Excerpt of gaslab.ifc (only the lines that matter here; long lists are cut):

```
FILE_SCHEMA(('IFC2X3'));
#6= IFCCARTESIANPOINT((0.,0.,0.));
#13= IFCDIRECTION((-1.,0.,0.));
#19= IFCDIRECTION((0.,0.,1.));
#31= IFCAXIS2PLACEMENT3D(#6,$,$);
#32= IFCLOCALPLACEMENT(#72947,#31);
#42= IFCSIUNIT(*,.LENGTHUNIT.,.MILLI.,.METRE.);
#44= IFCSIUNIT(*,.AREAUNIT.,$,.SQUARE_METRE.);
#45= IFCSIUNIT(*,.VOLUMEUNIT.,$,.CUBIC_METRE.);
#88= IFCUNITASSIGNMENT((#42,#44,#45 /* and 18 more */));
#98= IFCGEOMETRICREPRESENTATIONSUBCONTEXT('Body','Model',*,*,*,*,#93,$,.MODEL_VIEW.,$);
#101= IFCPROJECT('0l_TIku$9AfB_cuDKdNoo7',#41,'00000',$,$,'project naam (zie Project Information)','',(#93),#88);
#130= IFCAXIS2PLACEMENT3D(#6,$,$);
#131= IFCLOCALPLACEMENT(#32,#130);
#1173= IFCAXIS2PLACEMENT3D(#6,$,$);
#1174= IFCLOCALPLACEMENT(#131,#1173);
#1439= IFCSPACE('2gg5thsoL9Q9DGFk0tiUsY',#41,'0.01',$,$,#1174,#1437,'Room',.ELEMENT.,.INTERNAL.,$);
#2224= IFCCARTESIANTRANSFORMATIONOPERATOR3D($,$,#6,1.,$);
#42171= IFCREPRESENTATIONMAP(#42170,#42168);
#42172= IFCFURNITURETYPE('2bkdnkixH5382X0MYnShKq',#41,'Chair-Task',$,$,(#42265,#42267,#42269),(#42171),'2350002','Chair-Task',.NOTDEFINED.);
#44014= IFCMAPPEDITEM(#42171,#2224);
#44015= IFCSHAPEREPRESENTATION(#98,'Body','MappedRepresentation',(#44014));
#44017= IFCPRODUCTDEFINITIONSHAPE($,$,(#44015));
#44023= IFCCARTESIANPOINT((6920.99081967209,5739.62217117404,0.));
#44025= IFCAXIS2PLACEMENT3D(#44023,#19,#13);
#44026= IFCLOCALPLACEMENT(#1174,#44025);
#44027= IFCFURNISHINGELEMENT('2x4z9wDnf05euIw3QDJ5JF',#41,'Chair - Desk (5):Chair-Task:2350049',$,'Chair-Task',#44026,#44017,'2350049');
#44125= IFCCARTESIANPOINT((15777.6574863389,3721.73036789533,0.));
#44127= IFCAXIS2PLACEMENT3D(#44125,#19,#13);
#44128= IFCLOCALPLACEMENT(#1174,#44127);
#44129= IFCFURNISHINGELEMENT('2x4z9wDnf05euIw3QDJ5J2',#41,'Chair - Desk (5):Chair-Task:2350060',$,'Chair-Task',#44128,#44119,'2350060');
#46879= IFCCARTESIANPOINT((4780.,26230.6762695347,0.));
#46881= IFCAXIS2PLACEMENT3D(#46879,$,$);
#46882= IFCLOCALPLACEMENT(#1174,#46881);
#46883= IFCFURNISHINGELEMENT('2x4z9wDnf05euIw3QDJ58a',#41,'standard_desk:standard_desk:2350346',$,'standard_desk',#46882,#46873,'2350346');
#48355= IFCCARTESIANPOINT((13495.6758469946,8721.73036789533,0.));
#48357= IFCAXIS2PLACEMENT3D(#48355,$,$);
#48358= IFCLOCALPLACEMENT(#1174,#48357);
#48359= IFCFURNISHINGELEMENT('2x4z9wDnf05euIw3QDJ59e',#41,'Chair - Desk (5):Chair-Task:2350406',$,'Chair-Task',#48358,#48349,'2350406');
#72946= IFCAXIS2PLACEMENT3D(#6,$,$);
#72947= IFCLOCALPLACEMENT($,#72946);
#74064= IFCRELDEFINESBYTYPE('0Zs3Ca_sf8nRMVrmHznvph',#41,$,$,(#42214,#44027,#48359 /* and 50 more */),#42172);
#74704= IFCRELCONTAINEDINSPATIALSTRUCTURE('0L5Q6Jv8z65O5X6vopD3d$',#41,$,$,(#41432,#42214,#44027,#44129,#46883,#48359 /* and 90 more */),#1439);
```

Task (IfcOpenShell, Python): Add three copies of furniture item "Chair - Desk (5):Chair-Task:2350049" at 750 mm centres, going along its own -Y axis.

```python
import ifcopenshell
import ifcopenshell.api.geometry
import ifcopenshell.api.root
import ifcopenshell.util.element
import ifcopenshell.util.placement

model = ifcopenshell.open("gaslab.ifc")


def reuse_history(source, copy):
    """copy_class also copies each property set's owner history, people and application; keep the originals."""
    for rel in copy.IsDefinedBy:
        if rel.is_a("IfcRelDefinesByProperties") and (history := rel.RelatingPropertyDefinition.OwnerHistory):
            rel.RelatingPropertyDefinition.OwnerHistory = source.OwnerHistory
            ifcopenshell.util.element.remove_deep2(model, history)


source = model.by_guid("2x4z9wDnf05euIw3QDJ5JF")
base = ifcopenshell.util.placement.get_local_placement(source.ObjectPlacement)
step = -base[:3, 1] * 750.0

for i in range(1, 4):
    copy = ifcopenshell.api.root.copy_class(model, product=source)
    copy.Representation = ifcopenshell.util.element.copy_deep(
        model, source.Representation, exclude=["IfcGeometricRepresentationContext", "IfcRepresentationMap"]
    )
    copy.Name = "Chair - Desk (5):Chair-Task"
    copy.Tag = None
    reuse_history(source, copy)
    matrix = base.copy()
    matrix[:3, 3] += i * step
    print("added at", matrix[:3, 3].round(3) + 0.0)
    ifcopenshell.api.geometry.edit_object_placement(model, product=copy, matrix=matrix, is_si=False)

model.write("gaslab-out.ifc")
```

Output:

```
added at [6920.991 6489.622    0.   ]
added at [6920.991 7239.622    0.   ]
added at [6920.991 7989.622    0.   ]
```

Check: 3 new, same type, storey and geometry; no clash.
